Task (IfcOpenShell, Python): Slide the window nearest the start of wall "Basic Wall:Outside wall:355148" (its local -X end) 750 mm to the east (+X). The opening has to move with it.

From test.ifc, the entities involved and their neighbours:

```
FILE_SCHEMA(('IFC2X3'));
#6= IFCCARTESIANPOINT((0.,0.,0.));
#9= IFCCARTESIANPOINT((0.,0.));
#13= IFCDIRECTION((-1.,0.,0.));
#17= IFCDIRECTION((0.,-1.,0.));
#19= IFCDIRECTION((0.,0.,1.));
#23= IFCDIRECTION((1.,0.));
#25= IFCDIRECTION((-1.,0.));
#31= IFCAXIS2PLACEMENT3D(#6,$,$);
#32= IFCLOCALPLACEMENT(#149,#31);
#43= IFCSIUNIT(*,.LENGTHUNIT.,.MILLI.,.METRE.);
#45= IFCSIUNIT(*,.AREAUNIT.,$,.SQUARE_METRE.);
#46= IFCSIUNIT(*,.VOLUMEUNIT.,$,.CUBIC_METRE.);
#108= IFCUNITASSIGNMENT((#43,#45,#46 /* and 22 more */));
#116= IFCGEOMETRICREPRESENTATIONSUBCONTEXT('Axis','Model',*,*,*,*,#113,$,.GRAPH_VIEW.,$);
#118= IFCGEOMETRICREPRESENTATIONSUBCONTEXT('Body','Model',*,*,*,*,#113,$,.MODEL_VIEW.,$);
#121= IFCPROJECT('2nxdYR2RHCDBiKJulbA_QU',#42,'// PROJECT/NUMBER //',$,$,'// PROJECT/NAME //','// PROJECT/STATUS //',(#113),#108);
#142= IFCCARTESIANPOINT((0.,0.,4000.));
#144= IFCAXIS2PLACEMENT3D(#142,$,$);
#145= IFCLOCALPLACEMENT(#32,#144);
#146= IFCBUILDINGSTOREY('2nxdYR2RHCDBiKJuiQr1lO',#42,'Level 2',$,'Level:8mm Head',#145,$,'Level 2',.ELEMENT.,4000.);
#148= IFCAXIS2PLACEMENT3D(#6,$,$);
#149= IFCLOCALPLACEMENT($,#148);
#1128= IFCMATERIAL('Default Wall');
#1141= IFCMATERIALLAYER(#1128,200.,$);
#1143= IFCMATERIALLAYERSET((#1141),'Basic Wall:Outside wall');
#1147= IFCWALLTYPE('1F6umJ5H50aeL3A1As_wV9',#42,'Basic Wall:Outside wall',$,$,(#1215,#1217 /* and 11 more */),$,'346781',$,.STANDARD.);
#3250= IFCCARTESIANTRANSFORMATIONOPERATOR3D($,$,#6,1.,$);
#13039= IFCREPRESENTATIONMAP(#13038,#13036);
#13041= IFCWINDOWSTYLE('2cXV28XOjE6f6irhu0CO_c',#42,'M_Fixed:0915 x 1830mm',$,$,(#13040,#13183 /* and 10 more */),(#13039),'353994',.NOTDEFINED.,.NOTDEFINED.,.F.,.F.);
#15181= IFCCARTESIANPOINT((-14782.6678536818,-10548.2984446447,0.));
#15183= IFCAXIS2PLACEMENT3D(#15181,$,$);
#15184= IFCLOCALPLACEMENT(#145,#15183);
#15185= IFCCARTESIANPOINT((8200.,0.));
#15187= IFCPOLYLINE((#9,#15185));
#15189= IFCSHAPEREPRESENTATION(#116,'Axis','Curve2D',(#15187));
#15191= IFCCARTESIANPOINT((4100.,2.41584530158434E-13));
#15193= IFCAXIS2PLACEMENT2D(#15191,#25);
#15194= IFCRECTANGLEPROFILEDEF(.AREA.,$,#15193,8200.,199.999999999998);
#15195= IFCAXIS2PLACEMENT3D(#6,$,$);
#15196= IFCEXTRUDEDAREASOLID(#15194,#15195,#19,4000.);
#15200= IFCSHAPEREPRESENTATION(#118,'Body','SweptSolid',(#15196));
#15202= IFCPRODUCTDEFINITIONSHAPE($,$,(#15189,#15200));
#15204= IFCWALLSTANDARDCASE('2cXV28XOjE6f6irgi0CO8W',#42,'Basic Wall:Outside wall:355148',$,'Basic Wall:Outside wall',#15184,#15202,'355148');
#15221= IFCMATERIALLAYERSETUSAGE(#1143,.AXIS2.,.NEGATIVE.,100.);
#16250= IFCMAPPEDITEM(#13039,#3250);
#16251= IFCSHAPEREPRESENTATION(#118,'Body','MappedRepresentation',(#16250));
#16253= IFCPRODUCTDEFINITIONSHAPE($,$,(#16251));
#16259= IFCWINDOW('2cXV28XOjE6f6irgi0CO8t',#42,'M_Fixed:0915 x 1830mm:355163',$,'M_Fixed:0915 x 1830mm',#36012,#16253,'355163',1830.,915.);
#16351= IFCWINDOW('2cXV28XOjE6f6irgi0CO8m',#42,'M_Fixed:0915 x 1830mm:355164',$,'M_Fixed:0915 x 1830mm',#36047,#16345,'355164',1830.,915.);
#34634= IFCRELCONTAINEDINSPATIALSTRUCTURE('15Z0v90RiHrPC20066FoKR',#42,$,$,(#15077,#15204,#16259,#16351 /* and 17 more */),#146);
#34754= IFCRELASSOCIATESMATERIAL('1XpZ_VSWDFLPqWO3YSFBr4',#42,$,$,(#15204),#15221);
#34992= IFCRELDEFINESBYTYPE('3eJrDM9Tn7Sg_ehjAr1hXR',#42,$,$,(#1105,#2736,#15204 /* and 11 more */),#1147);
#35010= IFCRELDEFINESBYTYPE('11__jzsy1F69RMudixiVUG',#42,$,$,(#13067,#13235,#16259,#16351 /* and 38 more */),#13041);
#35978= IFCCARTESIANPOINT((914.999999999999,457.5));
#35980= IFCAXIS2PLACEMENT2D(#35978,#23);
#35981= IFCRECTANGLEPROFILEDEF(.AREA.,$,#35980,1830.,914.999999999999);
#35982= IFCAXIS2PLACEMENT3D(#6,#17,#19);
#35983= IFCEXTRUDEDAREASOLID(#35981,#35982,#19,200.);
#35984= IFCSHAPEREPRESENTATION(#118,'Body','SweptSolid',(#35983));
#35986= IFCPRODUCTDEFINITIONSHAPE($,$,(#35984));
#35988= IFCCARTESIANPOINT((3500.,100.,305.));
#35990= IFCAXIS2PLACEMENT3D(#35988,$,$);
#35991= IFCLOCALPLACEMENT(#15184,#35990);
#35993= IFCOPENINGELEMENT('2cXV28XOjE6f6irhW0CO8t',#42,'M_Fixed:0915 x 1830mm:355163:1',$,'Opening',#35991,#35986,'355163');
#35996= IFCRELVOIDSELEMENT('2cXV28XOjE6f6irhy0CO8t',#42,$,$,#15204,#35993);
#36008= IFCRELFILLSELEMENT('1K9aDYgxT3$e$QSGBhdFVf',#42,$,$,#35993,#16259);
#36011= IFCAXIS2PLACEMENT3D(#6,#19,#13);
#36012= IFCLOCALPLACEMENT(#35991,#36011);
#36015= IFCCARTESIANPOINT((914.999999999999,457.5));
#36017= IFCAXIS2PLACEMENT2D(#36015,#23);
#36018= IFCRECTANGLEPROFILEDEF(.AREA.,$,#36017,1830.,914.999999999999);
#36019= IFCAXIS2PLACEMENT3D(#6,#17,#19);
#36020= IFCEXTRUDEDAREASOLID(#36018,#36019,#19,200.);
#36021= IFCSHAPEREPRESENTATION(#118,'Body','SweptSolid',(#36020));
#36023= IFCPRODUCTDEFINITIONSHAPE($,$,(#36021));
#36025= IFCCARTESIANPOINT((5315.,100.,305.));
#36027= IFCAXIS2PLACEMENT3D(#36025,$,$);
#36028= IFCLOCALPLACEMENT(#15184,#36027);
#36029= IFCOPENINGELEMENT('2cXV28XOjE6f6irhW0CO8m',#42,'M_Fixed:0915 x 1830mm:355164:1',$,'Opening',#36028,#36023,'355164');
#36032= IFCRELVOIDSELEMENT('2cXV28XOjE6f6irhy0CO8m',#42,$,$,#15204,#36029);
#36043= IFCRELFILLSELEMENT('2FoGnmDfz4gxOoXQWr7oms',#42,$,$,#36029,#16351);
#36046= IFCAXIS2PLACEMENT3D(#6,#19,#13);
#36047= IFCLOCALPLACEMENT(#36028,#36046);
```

```python
import ifcopenshell
import ifcopenshell.api.geometry
import ifcopenshell.util.placement
import ifcopenshell.util.unit

model = ifcopenshell.open("test.ifc")
unit_scale = ifcopenshell.util.unit.calculate_unit_scale(model)

window = model.by_guid("2cXV28XOjE6f6irgi0CO8t")
opening = window.FillsVoids[0].RelatingOpeningElement
wall = opening.VoidsElements[0].RelatingBuildingElement

wall_matrix = ifcopenshell.util.placement.get_local_placement(wall.ObjectPlacement)
shift = wall_matrix[:3, 0] * 0.75 / unit_scale
before = ifcopenshell.util.placement.get_local_placement(window.ObjectPlacement)[:3, 3].copy()

# The window is placed relative to its opening, so it follows when the opening moves.
matrix = ifcopenshell.util.placement.get_local_placement(opening.ObjectPlacement)
matrix[:3, 3] += shift
ifcopenshell.api.geometry.edit_object_placement(
    model, product=opening, matrix=matrix, is_si=False, should_transform_children=True
)

after = ifcopenshell.util.placement.get_local_placement(window.ObjectPlacement)[:3, 3]
print("window moved by", (after - before).round(3) + 0.0)

model.write("test-out.ifc")
```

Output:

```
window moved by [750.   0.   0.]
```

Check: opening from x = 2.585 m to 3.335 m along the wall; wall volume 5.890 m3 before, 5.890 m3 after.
